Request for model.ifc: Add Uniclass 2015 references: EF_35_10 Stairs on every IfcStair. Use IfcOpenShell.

First a look at what the model holds.

```python
import ifcopenshell

model = ifcopenshell.open("model.ifc")
print(model.schema)
print("classifications:", [c.Name for c in model.by_type("IfcClassification")])
for ifc_class in ("IfcDoor", "IfcRoof", "IfcStair", "IfcWall", "IfcWindow"):
    print(ifc_class, len(model.by_type(ifc_class)))
```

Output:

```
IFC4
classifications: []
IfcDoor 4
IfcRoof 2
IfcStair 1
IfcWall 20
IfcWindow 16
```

```python
import ifcopenshell
import ifcopenshell.api.classification

model = ifcopenshell.open("model.ifc")

system = ifcopenshell.api.classification.add_classification(model, classification="Uniclass 2015")

codes = {
    "IfcStair": ("EF_35_10", "Stairs"),
}
for ifc_class, (code, name) in codes.items():
    products = model.by_type(ifc_class)
    ifcopenshell.api.classification.add_reference(
        model, products=products, classification=system, identification=code, name=name
    )
    print(code, len(products))

model.write("model_updated.ifc")
```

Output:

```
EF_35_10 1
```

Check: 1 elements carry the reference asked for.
